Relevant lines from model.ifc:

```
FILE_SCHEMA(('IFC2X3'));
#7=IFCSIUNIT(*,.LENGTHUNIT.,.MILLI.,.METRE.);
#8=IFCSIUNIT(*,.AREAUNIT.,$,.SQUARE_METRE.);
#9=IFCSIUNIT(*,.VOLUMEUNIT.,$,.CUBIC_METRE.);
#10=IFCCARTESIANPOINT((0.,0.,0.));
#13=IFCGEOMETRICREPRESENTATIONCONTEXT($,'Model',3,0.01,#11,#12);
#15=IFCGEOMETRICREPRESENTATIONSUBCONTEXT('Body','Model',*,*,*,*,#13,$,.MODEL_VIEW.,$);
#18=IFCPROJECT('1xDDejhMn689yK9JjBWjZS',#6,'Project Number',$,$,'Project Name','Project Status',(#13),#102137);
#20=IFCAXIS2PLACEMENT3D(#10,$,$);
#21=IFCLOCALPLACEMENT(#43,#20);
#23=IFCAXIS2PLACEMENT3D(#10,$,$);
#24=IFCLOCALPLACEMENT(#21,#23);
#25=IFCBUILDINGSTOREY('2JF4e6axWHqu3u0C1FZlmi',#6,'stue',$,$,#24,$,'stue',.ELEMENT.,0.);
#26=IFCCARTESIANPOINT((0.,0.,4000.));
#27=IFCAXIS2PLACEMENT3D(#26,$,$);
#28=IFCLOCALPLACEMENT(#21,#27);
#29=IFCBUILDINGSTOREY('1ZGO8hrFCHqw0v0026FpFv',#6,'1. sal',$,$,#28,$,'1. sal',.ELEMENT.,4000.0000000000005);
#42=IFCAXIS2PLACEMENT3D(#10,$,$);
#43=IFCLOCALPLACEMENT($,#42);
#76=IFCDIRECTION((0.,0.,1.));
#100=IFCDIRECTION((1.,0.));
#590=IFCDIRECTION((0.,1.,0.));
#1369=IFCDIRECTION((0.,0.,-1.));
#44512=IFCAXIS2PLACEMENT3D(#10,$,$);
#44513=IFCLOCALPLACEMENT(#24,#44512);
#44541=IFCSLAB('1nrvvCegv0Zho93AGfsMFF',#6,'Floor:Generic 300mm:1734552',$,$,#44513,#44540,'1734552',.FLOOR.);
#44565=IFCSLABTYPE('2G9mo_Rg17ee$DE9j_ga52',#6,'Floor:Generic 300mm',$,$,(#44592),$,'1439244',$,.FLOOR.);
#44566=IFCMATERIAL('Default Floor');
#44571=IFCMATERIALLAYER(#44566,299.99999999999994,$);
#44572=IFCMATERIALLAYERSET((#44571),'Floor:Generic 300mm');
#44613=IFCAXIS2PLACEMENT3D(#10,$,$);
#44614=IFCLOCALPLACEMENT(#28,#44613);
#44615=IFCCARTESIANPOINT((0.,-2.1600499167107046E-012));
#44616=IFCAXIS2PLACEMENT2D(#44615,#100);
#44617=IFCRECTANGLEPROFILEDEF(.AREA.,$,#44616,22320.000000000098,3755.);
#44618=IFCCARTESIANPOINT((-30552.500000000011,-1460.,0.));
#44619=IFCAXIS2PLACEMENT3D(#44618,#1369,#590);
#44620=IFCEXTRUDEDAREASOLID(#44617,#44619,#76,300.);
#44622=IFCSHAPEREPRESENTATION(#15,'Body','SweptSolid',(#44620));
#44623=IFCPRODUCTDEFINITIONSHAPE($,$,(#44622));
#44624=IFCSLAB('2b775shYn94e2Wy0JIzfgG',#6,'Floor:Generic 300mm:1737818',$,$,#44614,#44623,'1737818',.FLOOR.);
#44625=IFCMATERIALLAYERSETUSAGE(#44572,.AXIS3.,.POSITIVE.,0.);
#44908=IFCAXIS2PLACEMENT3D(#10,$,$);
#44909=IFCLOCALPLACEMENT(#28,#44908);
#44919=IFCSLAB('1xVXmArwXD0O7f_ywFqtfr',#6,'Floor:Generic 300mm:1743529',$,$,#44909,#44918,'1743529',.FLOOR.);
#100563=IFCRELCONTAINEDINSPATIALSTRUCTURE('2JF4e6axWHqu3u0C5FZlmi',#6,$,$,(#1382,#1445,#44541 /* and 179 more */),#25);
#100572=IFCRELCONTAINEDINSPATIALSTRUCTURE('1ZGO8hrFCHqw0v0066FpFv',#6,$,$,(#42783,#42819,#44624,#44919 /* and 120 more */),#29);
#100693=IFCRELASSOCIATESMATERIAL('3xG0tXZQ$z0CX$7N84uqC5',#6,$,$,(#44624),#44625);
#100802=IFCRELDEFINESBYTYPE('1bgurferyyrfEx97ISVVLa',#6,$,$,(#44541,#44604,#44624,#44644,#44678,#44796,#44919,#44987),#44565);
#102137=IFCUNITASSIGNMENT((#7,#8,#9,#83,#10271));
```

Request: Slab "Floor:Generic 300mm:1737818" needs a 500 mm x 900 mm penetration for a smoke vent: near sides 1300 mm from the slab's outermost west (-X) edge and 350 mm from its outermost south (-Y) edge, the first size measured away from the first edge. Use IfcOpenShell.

```python
import numpy as np
import ifcopenshell
import ifcopenshell.api.feature
import ifcopenshell.api.geometry
import ifcopenshell.api.root
import ifcopenshell.geom
import ifcopenshell.util.placement
import ifcopenshell.util.representation
import ifcopenshell.util.shape
import ifcopenshell.util.unit

model = ifcopenshell.open("model.ifc")
unit_scale = ifcopenshell.util.unit.calculate_unit_scale(model)
settings = ifcopenshell.geom.settings()


def volume(element):
    """Net volume in cubic metres, openings subtracted."""
    shape = ifcopenshell.geom.create_shape(settings, element)
    return ifcopenshell.util.shape.get_volume(shape.geometry)


slab = model.by_guid("2b775shYn94e2Wy0JIzfgG")
before = volume(slab)

# Extent in the slab's own axes, in metres. The edges named are its -X and -Y sides.
slab_shape = ifcopenshell.geom.create_shape(settings, slab)
vertices = ifcopenshell.util.shape.get_vertices(slab_shape.geometry)
x_min, y_min, bottom = vertices.min(axis=0)
top = vertices[:, 2].max()

opening = ifcopenshell.api.root.create_entity(model, ifc_class="IfcOpeningElement", name="Smoke vent opening")
context = ifcopenshell.util.representation.get_context(model, "Model", "Body", "MODEL_VIEW")
width, depth = 0.5, 0.9
outline = [(0.0, 0.0), (width, 0.0), (width, depth), (0.0, depth), (0.0, 0.0)]
# Overshoot both faces by 50 mm so the cut is clean.
shape = ifcopenshell.api.geometry.add_slab_representation(
    model, context=context, depth=top - bottom + 0.1, polyline=outline
)
ifcopenshell.api.geometry.assign_representation(model, product=opening, representation=shape)

matrix = ifcopenshell.util.placement.get_local_placement(slab.ObjectPlacement)
matrix[:, 3] = matrix @ np.append(np.array([x_min + 1.3, y_min + 0.35, bottom - 0.05]) / unit_scale, 1.0)
ifcopenshell.api.geometry.edit_object_placement(model, product=opening, matrix=matrix, is_si=False)
ifcopenshell.api.feature.add_feature(model, feature=opening, element=slab)

after = volume(slab)

print(f"slab volume {before:.3f} -> {after:.3f} m3")

model.write("model-out.ifc")
```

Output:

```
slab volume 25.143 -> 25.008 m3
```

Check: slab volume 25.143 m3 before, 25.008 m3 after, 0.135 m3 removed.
